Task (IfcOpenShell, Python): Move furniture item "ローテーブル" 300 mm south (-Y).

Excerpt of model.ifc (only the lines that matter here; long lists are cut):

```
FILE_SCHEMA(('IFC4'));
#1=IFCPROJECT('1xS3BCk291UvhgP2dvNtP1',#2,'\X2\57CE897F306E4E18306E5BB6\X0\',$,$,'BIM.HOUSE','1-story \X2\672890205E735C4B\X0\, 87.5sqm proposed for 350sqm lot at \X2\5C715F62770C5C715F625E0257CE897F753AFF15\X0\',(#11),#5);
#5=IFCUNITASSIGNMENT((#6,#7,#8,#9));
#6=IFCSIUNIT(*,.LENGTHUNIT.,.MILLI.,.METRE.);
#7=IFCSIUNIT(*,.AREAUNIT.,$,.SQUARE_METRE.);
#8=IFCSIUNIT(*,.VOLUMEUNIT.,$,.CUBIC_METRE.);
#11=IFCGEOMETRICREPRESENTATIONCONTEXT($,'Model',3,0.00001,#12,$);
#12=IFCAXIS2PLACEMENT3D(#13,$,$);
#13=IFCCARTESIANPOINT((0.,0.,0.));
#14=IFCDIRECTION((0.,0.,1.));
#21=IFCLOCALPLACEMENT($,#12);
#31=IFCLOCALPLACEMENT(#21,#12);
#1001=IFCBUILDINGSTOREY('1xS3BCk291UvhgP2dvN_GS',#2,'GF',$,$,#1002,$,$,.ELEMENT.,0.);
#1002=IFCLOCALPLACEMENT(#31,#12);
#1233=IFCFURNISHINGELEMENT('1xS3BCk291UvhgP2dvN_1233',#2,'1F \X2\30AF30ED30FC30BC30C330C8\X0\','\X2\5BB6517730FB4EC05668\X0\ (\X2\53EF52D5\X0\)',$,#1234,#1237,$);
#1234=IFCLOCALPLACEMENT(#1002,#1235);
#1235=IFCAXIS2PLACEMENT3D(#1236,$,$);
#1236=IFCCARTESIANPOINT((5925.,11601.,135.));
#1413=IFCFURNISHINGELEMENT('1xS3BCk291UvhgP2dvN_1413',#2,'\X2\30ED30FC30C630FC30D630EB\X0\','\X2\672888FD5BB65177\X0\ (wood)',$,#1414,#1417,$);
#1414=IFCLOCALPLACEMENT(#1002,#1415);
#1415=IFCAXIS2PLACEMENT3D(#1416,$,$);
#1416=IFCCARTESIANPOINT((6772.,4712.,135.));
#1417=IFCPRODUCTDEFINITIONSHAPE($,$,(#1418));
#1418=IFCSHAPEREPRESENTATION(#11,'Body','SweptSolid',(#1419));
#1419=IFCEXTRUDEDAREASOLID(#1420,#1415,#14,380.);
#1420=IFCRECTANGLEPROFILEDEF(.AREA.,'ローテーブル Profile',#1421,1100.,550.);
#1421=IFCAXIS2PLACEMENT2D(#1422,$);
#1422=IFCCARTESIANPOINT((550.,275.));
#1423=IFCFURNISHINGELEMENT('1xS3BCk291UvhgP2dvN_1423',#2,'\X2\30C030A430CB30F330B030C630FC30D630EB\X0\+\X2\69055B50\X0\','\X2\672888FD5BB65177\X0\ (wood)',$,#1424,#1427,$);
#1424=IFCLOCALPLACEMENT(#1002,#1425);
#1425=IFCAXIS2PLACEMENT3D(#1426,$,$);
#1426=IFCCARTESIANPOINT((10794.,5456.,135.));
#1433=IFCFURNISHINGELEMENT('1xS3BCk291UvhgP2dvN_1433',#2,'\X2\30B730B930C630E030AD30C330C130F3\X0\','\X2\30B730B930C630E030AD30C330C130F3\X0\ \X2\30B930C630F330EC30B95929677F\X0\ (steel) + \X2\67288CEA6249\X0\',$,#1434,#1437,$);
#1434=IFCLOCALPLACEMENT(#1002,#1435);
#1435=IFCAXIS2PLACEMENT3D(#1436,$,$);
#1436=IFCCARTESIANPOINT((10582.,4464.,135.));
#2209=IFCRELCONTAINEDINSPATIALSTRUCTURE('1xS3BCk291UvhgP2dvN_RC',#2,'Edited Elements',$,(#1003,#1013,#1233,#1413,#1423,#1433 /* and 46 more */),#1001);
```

```python
import ifcopenshell
import ifcopenshell.api.geometry
import ifcopenshell.util.placement

model = ifcopenshell.open("model.ifc")

item = model.by_guid("1xS3BCk291UvhgP2dvN_1413")
matrix = ifcopenshell.util.placement.get_local_placement(item.ObjectPlacement)
matrix[1, 3] -= 300.0
ifcopenshell.api.geometry.edit_object_placement(model, product=item, matrix=matrix, is_si=False)

print(ifcopenshell.util.placement.get_local_placement(item.ObjectPlacement).round(3) + 0.0)

model.write("model_rev.ifc")
```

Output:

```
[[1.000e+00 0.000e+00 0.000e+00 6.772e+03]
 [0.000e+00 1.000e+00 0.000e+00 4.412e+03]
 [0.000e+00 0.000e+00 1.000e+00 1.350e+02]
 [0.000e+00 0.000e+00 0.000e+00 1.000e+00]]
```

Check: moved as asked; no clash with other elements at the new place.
